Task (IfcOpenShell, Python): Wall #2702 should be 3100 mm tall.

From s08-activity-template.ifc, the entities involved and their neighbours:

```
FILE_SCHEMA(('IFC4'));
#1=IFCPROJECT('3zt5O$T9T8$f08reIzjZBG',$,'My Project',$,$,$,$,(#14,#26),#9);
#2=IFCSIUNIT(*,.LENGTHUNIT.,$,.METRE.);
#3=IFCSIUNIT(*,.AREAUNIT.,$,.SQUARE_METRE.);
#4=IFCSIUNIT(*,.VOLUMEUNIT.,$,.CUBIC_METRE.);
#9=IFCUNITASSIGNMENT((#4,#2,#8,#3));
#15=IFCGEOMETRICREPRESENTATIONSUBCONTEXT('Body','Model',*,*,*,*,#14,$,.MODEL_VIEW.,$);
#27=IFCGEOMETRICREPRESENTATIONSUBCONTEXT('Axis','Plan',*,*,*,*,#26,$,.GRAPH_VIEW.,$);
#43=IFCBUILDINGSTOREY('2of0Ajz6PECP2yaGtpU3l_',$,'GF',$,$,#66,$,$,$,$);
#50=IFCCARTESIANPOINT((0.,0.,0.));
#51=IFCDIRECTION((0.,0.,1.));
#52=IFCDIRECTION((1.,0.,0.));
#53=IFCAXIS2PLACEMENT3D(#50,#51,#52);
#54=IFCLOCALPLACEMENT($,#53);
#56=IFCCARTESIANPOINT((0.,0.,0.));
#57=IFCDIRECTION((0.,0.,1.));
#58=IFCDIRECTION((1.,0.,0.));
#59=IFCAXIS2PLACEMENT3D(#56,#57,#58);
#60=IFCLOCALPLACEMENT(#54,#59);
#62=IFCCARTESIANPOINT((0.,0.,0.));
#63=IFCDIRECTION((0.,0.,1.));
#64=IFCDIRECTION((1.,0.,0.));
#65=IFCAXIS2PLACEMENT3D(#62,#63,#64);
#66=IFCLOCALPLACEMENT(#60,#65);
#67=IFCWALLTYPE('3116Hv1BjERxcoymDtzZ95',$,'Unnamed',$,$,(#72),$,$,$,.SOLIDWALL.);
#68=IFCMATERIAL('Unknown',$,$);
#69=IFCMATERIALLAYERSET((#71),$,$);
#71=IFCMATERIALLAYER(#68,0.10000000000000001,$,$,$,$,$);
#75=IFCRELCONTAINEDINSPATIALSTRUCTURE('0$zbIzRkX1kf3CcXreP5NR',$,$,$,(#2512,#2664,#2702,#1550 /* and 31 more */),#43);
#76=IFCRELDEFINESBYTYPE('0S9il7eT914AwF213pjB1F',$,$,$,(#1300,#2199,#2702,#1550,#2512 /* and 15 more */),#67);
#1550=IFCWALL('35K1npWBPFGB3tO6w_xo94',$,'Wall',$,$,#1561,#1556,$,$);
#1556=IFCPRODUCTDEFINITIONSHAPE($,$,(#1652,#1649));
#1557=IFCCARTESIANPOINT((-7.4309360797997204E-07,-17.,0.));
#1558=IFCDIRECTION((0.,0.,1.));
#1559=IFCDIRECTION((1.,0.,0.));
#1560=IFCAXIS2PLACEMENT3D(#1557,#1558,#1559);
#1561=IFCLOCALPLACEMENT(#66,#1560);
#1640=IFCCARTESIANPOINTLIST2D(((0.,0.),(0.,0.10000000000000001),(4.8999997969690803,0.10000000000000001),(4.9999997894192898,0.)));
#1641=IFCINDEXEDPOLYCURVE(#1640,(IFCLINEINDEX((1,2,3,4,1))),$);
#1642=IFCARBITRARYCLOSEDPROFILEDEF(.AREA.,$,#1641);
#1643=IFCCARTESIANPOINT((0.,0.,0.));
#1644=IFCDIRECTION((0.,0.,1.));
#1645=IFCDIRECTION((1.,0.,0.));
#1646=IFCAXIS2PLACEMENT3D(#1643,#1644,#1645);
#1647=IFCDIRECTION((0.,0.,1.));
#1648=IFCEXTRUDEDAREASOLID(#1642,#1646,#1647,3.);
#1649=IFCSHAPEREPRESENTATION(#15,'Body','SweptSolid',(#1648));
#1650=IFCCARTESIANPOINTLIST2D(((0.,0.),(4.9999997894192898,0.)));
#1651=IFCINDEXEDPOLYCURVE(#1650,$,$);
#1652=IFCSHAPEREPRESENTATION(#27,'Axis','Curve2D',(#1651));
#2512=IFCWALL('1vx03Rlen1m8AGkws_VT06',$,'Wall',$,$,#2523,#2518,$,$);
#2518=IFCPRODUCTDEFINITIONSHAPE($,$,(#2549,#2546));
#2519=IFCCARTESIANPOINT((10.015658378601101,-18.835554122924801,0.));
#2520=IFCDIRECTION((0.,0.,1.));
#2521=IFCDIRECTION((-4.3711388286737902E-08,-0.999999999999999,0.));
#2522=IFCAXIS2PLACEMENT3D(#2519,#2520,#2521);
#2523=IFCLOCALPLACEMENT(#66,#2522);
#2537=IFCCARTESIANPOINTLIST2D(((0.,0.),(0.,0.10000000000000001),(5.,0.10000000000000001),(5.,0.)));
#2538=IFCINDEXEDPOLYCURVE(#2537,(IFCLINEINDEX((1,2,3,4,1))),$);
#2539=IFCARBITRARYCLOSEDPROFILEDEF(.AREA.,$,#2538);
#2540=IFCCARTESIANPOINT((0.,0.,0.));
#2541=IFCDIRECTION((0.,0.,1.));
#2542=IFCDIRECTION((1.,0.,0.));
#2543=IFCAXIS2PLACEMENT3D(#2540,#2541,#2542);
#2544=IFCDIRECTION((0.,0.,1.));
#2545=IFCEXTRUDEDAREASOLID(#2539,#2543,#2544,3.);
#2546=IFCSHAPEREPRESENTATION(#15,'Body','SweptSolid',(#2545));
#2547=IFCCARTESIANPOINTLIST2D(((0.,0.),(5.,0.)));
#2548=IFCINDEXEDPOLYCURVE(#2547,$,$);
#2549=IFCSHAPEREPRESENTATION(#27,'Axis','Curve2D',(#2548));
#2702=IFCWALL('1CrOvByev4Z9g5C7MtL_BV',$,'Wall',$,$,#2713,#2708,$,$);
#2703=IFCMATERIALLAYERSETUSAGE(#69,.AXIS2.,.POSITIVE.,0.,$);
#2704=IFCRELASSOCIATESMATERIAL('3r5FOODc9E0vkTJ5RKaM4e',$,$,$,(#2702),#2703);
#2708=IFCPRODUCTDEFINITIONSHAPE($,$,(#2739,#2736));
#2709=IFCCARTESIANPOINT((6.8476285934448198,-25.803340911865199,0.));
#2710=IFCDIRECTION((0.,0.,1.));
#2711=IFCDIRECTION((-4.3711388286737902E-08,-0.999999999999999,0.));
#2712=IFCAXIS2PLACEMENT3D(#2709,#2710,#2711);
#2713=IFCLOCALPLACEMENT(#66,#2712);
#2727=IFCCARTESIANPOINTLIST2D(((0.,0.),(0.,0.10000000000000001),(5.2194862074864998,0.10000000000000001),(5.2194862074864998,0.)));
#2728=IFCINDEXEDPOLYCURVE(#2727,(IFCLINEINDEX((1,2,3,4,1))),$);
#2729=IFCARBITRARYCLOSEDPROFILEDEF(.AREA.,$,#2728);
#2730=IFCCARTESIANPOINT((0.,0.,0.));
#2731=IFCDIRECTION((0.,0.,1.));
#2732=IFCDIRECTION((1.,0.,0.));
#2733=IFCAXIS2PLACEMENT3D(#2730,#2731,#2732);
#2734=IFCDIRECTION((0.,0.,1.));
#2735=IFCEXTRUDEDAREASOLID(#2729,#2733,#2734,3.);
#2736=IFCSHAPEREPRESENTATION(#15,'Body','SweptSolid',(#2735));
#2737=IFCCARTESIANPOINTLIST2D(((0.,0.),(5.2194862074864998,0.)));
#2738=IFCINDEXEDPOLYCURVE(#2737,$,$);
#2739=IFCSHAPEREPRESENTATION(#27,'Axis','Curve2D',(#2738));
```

```python
import ifcopenshell
import ifcopenshell.geom
import ifcopenshell.util.representation
import ifcopenshell.util.shape
import ifcopenshell.util.unit

model = ifcopenshell.open("s08-activity-template.ifc")
unit_scale = ifcopenshell.util.unit.calculate_unit_scale(model)
settings = ifcopenshell.geom.settings()


def volume(element):
    """Net volume in cubic metres, openings subtracted."""
    shape = ifcopenshell.geom.create_shape(settings, element)
    return ifcopenshell.util.shape.get_volume(shape.geometry)


wall = model.by_id(2702)
before = volume(wall)

body = ifcopenshell.util.representation.get_representation(wall, "Model", "Body")
solid = body.Items[0]
old_height = solid.Depth
solid.Depth = 3.1 / unit_scale
after = volume(wall)

print(f"height {old_height:g} -> {solid.Depth:g}, volume {before:.3f} -> {after:.3f} m3")

model.write("s08-activity-template_v2.ifc")
```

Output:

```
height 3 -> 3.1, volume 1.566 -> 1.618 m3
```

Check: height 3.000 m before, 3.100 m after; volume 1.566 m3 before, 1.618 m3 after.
